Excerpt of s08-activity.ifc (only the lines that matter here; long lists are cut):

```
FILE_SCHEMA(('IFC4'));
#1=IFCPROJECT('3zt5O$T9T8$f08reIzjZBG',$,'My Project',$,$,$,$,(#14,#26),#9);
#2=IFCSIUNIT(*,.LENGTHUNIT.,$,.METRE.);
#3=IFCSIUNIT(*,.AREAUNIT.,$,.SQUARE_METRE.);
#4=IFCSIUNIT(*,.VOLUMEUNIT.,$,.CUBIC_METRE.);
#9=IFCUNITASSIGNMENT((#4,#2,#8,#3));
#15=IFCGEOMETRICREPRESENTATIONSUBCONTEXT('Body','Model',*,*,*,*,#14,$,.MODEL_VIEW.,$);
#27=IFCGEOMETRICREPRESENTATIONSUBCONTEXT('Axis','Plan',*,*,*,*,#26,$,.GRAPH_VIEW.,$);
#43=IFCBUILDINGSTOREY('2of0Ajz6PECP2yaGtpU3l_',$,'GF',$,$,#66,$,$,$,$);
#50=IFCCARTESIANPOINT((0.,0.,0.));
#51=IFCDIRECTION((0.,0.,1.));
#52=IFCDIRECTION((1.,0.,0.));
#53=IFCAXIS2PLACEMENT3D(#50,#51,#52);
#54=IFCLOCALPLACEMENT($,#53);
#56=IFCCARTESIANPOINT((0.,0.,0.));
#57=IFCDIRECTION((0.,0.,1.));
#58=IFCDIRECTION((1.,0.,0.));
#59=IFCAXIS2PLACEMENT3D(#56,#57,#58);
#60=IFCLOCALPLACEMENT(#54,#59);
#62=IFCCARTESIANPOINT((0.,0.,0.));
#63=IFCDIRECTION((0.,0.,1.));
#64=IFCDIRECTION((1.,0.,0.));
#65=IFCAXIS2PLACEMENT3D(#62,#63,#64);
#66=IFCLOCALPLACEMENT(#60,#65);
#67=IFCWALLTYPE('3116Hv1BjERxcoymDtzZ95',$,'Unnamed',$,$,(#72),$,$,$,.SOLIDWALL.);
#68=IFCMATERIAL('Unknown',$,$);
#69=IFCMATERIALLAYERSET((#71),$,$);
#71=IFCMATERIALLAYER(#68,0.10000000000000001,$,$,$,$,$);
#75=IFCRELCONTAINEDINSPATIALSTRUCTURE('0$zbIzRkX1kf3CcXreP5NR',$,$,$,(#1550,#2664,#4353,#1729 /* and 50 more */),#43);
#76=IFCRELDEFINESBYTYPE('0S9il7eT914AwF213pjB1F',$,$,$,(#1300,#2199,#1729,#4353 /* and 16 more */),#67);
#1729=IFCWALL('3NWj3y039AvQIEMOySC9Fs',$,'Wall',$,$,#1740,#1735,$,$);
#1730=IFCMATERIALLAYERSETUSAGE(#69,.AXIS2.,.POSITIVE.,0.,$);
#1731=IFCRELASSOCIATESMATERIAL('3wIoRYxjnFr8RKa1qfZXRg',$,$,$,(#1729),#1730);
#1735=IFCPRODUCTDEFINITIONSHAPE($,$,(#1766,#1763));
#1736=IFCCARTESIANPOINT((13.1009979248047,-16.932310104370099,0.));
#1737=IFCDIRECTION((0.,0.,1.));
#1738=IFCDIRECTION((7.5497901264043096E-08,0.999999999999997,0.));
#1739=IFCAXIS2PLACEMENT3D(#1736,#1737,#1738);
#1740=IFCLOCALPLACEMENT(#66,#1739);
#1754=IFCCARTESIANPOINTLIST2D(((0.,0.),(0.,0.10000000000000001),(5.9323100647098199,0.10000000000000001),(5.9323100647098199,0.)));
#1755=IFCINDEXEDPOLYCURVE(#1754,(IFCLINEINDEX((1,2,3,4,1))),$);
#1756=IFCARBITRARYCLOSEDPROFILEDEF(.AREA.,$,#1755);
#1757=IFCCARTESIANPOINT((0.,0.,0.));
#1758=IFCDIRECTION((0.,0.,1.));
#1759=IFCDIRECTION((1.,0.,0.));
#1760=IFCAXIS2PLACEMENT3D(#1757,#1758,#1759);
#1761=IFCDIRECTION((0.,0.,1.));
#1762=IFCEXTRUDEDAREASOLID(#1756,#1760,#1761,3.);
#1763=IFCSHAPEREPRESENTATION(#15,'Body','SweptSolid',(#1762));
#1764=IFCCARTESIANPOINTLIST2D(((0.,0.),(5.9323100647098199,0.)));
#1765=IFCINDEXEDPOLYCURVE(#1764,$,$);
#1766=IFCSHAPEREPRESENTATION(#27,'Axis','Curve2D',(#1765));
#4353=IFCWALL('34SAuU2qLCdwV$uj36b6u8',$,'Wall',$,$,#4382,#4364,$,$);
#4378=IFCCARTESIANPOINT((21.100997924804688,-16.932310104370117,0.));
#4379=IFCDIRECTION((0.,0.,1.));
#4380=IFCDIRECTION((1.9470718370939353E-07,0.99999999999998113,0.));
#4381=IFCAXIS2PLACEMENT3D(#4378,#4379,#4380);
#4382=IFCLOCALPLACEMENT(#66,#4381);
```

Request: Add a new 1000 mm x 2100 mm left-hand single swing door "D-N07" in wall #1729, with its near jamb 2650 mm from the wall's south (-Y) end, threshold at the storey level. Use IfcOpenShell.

```python
import numpy as np
import ifcopenshell
import ifcopenshell.api.feature
import ifcopenshell.api.geometry
import ifcopenshell.api.root
import ifcopenshell.api.spatial
import ifcopenshell.geom
import ifcopenshell.util.element
import ifcopenshell.util.placement
import ifcopenshell.util.representation
import ifcopenshell.util.shape
import ifcopenshell.util.unit

model = ifcopenshell.open("s08-activity.ifc")
unit_scale = ifcopenshell.util.unit.calculate_unit_scale(model)
settings = ifcopenshell.geom.settings()


def volume(element):
    """Net volume in cubic metres, openings subtracted."""
    shape = ifcopenshell.geom.create_shape(settings, element)
    return ifcopenshell.util.shape.get_volume(shape.geometry)


wall = model.by_guid("3NWj3y039AvQIEMOySC9Fs")
storey = ifcopenshell.util.element.get_container(wall, ifc_class="IfcBuildingStorey")
context = ifcopenshell.util.representation.get_context(model, "Model", "Body", "MODEL_VIEW")
before = volume(wall)

width, height, from_end, sill = 1, 2.1, 2.65, 0.0  # metres

# The wall runs along its own X axis, and the end named is its -X end.
wall_shape = ifcopenshell.geom.create_shape(settings, wall)
x, y, z = ifcopenshell.util.shape.get_vertices(wall_shape.geometry).T
start = x.min() + from_end
face, thickness = float(y.min()), float(y.max() - y.min())
wall_matrix = ifcopenshell.util.placement.get_local_placement(wall.ObjectPlacement)
level = ifcopenshell.util.placement.get_local_placement(storey.ObjectPlacement)[2, 3]


def in_wall(x, y):
    """Placement at x, y metres in the wall's axes, at sill height."""
    matrix = wall_matrix.copy()
    matrix[:, 3] = wall_matrix @ np.array([x / unit_scale, y / unit_scale, 0.0, 1.0])
    matrix[2, 3] = level + sill / unit_scale
    return matrix


# Opening: a box that overshoots both wall faces by 50 mm.
opening = ifcopenshell.api.root.create_entity(model, ifc_class="IfcOpeningElement", predefined_type="OPENING")
box = ifcopenshell.api.geometry.add_wall_representation(
    model, context=context, length=width, height=height, thickness=thickness + 0.1
)
ifcopenshell.api.geometry.assign_representation(model, product=opening, representation=box)
ifcopenshell.api.geometry.edit_object_placement(model, product=opening, matrix=in_wall(start, face - 0.05), is_si=False)
ifcopenshell.api.feature.add_feature(model, feature=opening, element=wall)

door = ifcopenshell.api.root.create_entity(model, ifc_class="IfcDoor", name="D-N07", predefined_type="DOOR")
door.OverallWidth, door.OverallHeight = width / unit_scale, height / unit_scale
door.OperationType = "SINGLE_SWING_LEFT"
body = ifcopenshell.api.geometry.add_door_representation(
    model,
    context=context,
    overall_width=door.OverallWidth,
    overall_height=door.OverallHeight,
    operation_type="SINGLE_SWING_LEFT",
    lining_properties={"LiningDepth": thickness / unit_scale, "ThresholdDepth": thickness / unit_scale},
)
ifcopenshell.api.geometry.assign_representation(model, product=door, representation=body)
ifcopenshell.api.spatial.assign_container(model, products=[door], relating_structure=storey)
ifcopenshell.api.feature.add_filling(model, opening=opening, element=door)

# The lining spans the wall, so the door starts at the wall face.
ifcopenshell.api.geometry.edit_object_placement(model, product=door, matrix=in_wall(start, face), is_si=False)

after = volume(wall)

print(f"wall volume {before:.3f} -> {after:.3f} m3")

model.write("s08-activity_updated.ifc")
```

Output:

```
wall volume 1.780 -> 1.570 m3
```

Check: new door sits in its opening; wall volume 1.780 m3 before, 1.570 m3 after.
